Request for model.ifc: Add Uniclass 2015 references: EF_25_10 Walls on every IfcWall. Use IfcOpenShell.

First a look at what the model holds.

```python
import ifcopenshell

model = ifcopenshell.open("model.ifc")
print(model.schema)
print("classifications:", [c.Name for c in model.by_type("IfcClassification")])
for ifc_class in ("IfcDoor", "IfcRoof", "IfcStair", "IfcWall", "IfcWindow"):
    print(ifc_class, len(model.by_type(ifc_class)))
```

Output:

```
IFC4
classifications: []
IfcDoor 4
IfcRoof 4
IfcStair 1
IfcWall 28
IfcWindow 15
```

```python
import ifcopenshell
import ifcopenshell.api.classification

model = ifcopenshell.open("model.ifc")

system = ifcopenshell.api.classification.add_classification(model, classification="Uniclass 2015")

codes = {
    "IfcWall": ("EF_25_10", "Walls"),
}
for ifc_class, (code, name) in codes.items():
    products = model.by_type(ifc_class)
    ifcopenshell.api.classification.add_reference(
        model, products=products, classification=system, identification=code, name=name
    )
    print(code, len(products))

model.write("model_updated.ifc")
```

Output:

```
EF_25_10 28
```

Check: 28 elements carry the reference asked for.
